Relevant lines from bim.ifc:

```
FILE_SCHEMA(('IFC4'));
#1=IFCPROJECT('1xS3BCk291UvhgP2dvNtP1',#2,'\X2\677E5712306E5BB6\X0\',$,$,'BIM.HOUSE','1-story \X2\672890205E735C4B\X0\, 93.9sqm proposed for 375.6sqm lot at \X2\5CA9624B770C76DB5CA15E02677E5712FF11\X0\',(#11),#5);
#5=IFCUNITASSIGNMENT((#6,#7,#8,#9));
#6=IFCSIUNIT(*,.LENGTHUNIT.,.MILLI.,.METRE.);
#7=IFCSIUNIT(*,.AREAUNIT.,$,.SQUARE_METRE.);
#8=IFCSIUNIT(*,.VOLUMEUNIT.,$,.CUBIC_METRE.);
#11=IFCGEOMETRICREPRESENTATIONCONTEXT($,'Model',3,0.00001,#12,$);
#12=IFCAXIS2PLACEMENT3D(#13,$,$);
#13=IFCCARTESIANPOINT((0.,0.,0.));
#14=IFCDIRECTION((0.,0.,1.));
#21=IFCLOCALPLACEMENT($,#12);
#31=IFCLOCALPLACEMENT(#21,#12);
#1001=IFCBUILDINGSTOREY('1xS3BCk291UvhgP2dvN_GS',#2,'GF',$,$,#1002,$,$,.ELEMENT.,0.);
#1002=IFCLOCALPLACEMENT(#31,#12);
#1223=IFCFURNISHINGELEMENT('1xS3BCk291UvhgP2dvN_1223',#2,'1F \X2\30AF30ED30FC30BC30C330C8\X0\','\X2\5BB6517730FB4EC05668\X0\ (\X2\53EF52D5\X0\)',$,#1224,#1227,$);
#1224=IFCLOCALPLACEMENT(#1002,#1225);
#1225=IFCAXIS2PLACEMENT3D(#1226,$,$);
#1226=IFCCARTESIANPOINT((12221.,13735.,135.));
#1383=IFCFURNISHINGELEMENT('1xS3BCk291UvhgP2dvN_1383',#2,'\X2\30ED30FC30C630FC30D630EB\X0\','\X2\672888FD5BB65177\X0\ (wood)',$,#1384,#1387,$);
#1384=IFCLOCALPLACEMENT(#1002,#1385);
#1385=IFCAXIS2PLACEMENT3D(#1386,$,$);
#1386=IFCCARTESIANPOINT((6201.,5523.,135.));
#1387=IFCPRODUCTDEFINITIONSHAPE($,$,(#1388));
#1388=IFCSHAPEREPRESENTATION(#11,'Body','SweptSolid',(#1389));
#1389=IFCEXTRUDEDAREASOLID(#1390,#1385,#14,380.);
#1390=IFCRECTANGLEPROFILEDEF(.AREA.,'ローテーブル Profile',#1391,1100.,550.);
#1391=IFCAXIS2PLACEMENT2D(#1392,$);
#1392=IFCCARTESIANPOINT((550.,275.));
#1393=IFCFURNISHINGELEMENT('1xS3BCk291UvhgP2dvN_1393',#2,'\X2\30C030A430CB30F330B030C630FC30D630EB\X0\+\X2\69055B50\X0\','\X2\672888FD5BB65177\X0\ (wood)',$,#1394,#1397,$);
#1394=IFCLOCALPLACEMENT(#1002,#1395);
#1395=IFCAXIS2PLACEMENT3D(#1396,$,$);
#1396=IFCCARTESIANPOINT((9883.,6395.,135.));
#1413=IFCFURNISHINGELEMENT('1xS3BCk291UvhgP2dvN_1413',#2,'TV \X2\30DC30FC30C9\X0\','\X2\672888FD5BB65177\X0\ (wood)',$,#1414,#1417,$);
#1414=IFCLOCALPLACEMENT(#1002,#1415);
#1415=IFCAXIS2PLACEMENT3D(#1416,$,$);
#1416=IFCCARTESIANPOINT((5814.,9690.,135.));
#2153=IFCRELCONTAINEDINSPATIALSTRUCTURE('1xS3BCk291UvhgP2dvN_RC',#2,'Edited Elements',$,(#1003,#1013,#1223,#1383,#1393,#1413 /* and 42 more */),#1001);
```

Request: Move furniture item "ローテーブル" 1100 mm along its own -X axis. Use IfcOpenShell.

```python
import ifcopenshell
import ifcopenshell.api.geometry
import ifcopenshell.util.placement
import ifcopenshell.util.unit

model = ifcopenshell.open("bim.ifc")
unit_scale = ifcopenshell.util.unit.calculate_unit_scale(model)

item = model.by_id(1383)
matrix = ifcopenshell.util.placement.get_local_placement(item.ObjectPlacement)
matrix[:3, 3] -= matrix[:3, 0] * 1.1 / unit_scale
ifcopenshell.api.geometry.edit_object_placement(model, product=item, matrix=matrix, is_si=False)

print(ifcopenshell.util.placement.get_local_placement(item.ObjectPlacement).round(3) + 0.0)

model.write("bim_edited.ifc")
```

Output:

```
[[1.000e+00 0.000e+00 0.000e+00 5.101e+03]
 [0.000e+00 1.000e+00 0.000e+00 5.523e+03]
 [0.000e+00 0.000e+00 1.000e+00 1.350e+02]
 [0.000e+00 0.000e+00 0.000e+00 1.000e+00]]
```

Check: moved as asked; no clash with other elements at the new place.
